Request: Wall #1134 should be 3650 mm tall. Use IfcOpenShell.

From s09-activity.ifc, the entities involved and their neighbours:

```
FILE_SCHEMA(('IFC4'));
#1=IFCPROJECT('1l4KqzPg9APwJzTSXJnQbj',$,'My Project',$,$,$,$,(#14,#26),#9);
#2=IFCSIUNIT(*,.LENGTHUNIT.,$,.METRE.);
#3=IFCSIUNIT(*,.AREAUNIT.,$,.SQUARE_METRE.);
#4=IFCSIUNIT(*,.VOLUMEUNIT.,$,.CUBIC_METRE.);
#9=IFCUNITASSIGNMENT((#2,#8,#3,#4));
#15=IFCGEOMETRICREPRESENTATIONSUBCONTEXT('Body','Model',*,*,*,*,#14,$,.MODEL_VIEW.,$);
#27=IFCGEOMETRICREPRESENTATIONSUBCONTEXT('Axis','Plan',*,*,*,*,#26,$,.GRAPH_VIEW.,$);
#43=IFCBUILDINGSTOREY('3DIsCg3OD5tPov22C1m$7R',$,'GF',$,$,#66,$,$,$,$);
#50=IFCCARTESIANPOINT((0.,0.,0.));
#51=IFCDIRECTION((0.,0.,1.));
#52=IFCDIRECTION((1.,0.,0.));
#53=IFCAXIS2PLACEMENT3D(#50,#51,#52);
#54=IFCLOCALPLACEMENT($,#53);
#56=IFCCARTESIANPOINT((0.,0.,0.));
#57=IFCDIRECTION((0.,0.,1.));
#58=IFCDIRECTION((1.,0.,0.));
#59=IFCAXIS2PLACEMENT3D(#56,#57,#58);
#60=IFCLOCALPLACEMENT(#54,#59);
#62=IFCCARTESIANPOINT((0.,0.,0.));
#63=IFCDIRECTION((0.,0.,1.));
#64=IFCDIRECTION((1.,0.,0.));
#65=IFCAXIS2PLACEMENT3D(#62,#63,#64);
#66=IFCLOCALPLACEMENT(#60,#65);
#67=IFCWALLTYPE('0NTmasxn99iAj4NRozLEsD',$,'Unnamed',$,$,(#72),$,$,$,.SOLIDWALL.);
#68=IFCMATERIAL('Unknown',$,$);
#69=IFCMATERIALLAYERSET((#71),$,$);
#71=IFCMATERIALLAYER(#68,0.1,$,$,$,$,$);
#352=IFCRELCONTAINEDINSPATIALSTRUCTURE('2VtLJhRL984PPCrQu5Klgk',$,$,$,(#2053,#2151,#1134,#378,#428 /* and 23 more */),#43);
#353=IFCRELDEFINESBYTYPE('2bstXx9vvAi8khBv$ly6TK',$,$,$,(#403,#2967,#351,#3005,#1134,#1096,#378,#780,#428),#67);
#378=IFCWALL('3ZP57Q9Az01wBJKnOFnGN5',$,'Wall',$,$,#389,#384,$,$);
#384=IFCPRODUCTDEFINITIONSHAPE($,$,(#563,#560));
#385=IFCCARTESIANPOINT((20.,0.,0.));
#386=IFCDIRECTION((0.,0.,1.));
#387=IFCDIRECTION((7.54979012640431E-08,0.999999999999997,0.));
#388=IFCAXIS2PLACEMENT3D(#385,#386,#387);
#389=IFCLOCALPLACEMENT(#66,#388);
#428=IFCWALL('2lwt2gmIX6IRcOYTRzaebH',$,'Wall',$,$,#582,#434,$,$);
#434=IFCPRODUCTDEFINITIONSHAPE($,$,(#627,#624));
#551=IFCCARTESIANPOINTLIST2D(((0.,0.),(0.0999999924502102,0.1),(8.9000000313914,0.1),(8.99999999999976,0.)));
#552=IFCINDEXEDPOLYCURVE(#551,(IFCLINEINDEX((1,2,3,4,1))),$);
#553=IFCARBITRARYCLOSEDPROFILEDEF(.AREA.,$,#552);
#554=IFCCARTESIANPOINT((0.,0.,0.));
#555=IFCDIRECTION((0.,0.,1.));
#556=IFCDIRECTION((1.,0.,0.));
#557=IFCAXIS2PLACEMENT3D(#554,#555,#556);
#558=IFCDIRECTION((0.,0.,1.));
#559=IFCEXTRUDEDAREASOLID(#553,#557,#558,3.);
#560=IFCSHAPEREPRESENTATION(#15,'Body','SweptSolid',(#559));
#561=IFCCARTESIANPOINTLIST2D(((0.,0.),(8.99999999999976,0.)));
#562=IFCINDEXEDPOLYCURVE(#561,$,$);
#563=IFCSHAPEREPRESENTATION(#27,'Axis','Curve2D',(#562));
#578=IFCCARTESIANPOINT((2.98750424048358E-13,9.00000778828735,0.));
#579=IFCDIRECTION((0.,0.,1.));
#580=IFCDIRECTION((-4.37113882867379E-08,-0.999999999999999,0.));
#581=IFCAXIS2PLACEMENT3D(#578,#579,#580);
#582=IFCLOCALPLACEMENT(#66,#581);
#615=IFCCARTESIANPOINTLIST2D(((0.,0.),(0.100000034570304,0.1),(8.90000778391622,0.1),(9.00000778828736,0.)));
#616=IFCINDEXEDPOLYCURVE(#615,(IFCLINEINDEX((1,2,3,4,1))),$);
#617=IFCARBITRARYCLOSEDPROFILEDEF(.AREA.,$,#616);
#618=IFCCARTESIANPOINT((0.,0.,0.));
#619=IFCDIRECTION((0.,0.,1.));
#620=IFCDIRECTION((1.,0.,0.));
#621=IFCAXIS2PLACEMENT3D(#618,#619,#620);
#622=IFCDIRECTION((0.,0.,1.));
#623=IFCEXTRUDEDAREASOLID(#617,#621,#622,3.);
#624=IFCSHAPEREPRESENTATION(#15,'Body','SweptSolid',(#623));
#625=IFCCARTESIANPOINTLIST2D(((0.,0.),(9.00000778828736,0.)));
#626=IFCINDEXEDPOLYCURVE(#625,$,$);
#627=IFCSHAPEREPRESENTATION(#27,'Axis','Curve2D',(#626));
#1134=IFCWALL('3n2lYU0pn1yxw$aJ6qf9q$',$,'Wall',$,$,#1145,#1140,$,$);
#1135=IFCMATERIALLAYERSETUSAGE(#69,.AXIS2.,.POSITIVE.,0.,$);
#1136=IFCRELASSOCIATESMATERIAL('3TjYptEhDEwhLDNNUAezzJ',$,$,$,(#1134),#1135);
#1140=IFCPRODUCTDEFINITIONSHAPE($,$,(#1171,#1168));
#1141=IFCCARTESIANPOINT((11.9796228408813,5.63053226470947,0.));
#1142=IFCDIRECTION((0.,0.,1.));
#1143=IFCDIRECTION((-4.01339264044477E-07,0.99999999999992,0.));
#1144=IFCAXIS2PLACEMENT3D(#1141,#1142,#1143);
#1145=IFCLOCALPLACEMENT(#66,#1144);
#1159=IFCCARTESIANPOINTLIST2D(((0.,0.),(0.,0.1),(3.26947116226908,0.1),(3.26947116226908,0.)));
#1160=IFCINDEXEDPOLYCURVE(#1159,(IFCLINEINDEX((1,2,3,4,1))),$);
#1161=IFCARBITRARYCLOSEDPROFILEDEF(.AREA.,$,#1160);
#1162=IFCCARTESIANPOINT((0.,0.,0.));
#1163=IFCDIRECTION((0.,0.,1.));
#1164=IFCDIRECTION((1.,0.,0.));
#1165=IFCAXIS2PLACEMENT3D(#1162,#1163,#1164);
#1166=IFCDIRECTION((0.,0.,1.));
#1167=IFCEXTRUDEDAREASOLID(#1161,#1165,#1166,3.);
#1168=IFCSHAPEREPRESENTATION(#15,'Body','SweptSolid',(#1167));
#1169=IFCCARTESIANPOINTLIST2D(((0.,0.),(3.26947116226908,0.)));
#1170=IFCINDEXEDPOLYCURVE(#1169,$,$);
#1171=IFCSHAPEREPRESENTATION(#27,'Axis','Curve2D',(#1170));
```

```python
import ifcopenshell
import ifcopenshell.geom
import ifcopenshell.util.representation
import ifcopenshell.util.shape
import ifcopenshell.util.unit

model = ifcopenshell.open("s09-activity.ifc")
unit_scale = ifcopenshell.util.unit.calculate_unit_scale(model)
settings = ifcopenshell.geom.settings()


def volume(element):
    """Net volume in cubic metres, openings subtracted."""
    shape = ifcopenshell.geom.create_shape(settings, element)
    return ifcopenshell.util.shape.get_volume(shape.geometry)


wall = model.by_guid("3n2lYU0pn1yxw$aJ6qf9q$")
before = volume(wall)

body = ifcopenshell.util.representation.get_representation(wall, "Model", "Body")
solid = body.Items[0]
old_height = solid.Depth
solid.Depth = 3.65 / unit_scale
after = volume(wall)

print(f"height {old_height:g} -> {solid.Depth:g}, volume {before:.3f} -> {after:.3f} m3")

model.write("s09-activity_edited.ifc")
```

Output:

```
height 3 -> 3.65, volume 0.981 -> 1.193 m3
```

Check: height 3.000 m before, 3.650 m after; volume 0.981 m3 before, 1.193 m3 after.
